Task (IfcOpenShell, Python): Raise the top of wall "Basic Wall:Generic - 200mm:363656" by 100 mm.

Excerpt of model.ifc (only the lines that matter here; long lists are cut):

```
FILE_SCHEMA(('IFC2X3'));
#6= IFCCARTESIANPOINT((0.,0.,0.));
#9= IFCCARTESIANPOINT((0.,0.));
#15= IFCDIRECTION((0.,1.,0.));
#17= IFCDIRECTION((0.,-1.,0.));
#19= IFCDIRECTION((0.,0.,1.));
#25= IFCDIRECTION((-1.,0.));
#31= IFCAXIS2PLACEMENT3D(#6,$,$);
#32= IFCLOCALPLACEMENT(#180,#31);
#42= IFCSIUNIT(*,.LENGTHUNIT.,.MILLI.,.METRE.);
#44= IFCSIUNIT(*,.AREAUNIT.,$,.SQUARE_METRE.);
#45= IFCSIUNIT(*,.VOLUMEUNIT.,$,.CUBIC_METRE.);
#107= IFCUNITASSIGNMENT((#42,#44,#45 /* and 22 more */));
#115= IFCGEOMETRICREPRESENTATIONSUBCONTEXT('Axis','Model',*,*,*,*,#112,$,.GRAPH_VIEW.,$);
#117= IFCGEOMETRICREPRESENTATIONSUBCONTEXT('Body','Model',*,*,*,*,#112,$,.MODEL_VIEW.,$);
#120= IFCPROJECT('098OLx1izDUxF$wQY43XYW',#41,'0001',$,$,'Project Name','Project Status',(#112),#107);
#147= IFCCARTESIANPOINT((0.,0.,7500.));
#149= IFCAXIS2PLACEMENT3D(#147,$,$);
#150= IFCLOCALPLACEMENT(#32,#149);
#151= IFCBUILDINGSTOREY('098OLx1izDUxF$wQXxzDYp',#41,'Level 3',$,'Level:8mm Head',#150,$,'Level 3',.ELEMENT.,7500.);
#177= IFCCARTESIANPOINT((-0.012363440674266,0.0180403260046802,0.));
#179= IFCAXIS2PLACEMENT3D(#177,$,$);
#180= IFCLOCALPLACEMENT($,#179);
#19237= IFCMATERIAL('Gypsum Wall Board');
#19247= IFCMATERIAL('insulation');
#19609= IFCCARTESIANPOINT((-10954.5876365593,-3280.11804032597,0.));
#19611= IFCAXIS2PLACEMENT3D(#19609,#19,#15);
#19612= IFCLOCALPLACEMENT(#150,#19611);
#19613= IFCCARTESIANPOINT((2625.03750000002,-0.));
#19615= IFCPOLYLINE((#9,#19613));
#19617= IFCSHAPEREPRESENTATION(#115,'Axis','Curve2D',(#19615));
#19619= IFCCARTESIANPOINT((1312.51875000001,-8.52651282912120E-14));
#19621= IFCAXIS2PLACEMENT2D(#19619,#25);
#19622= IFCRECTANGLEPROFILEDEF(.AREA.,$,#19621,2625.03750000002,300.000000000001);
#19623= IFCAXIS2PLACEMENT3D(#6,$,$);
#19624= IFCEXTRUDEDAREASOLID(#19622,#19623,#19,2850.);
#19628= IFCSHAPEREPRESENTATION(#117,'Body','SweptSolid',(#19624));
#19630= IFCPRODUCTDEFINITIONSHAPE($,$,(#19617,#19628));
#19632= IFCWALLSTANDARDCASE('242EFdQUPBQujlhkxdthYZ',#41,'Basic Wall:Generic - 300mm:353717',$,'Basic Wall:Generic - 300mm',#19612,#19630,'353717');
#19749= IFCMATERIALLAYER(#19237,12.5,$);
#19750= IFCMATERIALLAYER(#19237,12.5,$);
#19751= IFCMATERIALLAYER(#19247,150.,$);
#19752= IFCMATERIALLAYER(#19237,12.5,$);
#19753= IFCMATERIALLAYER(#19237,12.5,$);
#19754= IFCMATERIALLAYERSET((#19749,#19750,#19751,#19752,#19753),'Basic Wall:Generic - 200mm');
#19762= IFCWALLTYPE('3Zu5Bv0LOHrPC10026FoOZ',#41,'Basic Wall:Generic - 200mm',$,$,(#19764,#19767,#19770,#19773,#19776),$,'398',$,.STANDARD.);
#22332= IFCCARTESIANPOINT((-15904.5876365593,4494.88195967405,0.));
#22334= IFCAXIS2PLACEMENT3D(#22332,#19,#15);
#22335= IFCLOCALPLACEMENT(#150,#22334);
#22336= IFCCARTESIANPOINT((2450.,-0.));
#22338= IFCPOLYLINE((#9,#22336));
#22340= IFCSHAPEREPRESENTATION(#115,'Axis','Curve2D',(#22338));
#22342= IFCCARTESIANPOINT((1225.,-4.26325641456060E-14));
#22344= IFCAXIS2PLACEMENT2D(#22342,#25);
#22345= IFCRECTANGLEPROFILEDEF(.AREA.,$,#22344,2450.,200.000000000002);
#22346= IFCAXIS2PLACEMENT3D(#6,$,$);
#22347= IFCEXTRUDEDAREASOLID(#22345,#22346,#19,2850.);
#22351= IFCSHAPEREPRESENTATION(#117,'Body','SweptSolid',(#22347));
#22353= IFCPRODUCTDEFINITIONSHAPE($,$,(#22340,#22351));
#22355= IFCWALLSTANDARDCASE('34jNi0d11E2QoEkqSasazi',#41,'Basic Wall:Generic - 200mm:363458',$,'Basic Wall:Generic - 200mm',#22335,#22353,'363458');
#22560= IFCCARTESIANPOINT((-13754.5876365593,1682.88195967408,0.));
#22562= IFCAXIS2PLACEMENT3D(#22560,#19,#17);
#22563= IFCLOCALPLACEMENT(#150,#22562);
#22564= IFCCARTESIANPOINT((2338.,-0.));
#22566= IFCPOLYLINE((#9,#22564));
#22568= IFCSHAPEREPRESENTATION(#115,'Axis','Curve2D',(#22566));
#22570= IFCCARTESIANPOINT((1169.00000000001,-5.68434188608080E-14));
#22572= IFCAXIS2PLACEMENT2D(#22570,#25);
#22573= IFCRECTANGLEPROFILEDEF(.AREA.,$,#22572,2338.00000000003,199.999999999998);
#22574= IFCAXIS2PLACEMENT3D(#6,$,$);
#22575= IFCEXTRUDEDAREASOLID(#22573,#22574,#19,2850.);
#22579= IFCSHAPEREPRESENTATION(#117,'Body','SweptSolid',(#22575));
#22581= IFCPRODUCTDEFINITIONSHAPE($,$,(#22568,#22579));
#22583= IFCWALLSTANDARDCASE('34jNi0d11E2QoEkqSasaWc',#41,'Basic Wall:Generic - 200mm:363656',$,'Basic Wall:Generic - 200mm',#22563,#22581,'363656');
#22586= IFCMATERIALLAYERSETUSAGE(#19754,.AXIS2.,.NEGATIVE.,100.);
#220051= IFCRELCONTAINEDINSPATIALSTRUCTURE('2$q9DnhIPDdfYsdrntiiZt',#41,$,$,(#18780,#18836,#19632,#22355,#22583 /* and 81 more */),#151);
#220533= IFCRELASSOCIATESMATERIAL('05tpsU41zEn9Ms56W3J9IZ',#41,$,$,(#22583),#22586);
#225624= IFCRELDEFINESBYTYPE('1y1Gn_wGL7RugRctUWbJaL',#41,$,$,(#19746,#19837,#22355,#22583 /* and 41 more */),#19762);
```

```python
import ifcopenshell
import ifcopenshell.geom
import ifcopenshell.util.representation
import ifcopenshell.util.shape

model = ifcopenshell.open("model.ifc")
settings = ifcopenshell.geom.settings()


def volume(element):
    """Net volume in cubic metres, openings subtracted."""
    shape = ifcopenshell.geom.create_shape(settings, element)
    return ifcopenshell.util.shape.get_volume(shape.geometry)


wall = model.by_guid("34jNi0d11E2QoEkqSasaWc")
before = volume(wall)

body = ifcopenshell.util.representation.get_representation(wall, "Model", "Body")
solid = body.Items[0]
old_height = solid.Depth
solid.Depth += 100.0
after = volume(wall)

print(f"height {old_height:g} -> {solid.Depth:g}, volume {before:.3f} -> {after:.3f} m3")

model.write("model_edited.ifc")
```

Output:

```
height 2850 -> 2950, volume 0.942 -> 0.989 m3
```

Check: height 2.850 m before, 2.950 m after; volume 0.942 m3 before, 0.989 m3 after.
